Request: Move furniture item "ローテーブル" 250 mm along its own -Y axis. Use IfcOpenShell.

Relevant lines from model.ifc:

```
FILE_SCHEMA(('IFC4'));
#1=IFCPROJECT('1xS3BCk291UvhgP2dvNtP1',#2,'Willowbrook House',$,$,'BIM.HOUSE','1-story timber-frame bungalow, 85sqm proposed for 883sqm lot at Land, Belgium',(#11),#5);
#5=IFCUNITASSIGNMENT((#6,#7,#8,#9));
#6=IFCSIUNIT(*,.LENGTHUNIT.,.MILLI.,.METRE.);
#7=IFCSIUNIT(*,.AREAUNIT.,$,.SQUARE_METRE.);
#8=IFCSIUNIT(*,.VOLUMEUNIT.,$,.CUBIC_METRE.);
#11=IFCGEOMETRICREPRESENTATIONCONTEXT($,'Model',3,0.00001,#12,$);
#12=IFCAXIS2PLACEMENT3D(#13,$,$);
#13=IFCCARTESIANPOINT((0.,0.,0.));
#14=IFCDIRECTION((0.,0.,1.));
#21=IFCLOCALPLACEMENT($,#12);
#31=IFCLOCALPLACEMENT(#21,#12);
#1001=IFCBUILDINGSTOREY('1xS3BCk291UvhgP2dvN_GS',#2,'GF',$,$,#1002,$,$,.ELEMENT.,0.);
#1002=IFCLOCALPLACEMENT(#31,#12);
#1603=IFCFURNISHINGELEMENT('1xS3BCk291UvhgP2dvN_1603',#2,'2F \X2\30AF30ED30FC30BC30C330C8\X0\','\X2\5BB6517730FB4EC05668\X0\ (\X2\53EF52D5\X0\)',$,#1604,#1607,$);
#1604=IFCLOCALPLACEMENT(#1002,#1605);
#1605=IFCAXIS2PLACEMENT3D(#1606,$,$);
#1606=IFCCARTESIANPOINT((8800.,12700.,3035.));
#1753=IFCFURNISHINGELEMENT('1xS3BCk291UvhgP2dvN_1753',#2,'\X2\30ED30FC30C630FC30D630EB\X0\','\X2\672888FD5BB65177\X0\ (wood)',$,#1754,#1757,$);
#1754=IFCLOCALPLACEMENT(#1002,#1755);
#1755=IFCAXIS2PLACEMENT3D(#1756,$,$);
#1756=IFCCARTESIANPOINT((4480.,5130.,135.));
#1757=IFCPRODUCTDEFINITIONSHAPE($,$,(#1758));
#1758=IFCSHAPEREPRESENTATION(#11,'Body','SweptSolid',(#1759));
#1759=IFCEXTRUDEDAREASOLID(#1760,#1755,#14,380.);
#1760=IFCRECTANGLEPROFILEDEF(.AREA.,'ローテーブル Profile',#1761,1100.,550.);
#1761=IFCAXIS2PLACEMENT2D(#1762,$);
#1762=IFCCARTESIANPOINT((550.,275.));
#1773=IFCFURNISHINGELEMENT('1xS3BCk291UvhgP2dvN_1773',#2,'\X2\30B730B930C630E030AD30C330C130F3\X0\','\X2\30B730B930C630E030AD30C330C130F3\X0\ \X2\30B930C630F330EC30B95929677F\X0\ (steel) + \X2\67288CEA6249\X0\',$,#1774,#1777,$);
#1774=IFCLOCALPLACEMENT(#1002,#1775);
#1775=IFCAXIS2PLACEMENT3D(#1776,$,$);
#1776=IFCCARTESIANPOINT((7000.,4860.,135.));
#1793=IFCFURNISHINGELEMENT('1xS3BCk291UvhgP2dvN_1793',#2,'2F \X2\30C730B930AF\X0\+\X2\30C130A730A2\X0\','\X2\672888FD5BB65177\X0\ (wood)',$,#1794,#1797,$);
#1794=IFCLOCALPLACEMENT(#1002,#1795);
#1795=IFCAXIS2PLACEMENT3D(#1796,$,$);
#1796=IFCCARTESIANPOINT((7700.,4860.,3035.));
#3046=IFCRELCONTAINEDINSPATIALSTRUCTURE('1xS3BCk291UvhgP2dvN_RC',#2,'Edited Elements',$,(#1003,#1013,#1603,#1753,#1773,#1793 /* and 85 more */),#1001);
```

```python
import ifcopenshell
import ifcopenshell.api.geometry
import ifcopenshell.util.placement

model = ifcopenshell.open("model.ifc")

item = model.by_id(1753)
matrix = ifcopenshell.util.placement.get_local_placement(item.ObjectPlacement)
matrix[:3, 3] -= matrix[:3, 1] * 250.0
ifcopenshell.api.geometry.edit_object_placement(model, product=item, matrix=matrix, is_si=False)

print(ifcopenshell.util.placement.get_local_placement(item.ObjectPlacement).round(3) + 0.0)

model.write("model_edited.ifc")
```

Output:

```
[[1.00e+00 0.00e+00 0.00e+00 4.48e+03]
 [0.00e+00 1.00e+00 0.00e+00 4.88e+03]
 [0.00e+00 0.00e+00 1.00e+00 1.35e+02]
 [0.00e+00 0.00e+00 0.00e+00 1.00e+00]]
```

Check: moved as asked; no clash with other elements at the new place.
